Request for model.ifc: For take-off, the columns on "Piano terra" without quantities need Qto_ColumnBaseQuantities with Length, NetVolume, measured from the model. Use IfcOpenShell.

First a look at what the model holds.

```python
import ifcopenshell
import ifcopenshell.util.element
import ifcopenshell.util.unit

model = ifcopenshell.open("model.ifc")
print(model.schema)
for unit_type in ("LENGTHUNIT", "AREAUNIT", "VOLUMEUNIT"):
    print(unit_type, ifcopenshell.util.unit.calculate_unit_scale(model, unit_type))
storey = next(s for s in model.by_type("IfcBuildingStorey") if s.Name == "Piano terra")
columns = [e for e in ifcopenshell.util.element.get_decomposition(storey) if e.is_a("IfcColumn")]
for e in sorted(columns, key=lambda e: e.id()):
    print(e.id(), e.is_a(), e.Name, list(ifcopenshell.util.element.get_psets(e, qtos_only=True)), sep=" | ")
```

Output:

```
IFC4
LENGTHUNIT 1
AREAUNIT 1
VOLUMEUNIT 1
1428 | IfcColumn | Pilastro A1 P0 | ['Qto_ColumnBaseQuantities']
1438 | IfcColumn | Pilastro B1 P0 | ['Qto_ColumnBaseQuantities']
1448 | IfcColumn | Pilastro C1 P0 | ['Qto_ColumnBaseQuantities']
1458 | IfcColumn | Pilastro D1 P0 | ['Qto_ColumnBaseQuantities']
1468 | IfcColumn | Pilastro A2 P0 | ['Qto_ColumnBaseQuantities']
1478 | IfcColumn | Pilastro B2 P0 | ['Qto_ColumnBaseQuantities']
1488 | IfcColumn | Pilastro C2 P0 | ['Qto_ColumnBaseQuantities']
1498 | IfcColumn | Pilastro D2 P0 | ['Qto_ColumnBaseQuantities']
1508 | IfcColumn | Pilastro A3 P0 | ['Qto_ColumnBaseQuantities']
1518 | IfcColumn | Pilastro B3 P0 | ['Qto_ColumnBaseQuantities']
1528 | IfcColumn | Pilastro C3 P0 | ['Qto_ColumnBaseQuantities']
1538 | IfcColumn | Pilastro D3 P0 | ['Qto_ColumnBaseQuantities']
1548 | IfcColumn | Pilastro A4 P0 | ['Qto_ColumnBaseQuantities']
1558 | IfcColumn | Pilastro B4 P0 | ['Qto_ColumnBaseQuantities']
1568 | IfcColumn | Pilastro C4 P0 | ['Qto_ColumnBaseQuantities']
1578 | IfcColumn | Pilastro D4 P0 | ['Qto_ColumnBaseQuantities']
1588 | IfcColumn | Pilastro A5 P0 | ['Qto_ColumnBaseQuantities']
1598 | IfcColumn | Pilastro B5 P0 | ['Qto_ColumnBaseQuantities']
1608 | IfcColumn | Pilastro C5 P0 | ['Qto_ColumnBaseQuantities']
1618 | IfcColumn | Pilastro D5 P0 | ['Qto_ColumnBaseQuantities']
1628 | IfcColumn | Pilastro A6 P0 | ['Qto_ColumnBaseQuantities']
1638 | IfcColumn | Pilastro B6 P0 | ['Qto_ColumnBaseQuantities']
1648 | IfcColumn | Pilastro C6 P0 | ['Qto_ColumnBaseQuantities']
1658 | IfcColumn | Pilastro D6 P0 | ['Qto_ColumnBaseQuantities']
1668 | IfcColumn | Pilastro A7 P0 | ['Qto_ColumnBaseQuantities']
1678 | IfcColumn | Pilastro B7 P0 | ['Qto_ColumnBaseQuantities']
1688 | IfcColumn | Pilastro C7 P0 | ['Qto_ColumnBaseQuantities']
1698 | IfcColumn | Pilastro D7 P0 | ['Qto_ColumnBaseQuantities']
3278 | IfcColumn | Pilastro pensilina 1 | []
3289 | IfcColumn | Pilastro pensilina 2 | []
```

```python
import ifcopenshell
import ifcopenshell.api.pset
import ifcopenshell.geom
import ifcopenshell.util.element
import ifcopenshell.util.shape
import ifcopenshell.util.unit

model = ifcopenshell.open("model.ifc")
unit_scale = ifcopenshell.util.unit.calculate_unit_scale(model)
volume_scale = ifcopenshell.util.unit.calculate_unit_scale(model, "VOLUMEUNIT")
settings = ifcopenshell.geom.settings()

storey = next(s for s in model.by_type("IfcBuildingStorey") if s.Name == "Piano terra")
columns = [e for e in ifcopenshell.util.element.get_decomposition(storey) if e.is_a("IfcColumn")]

for e in sorted(columns, key=lambda e: e.id()):
    if ifcopenshell.util.element.get_psets(e, qtos_only=True, should_inherit=False):
        continue
    # Geometry comes back in metres, in the element's own axes.
    shape = ifcopenshell.geom.create_shape(settings, e)
    values = {
        "Length": ifcopenshell.util.shape.get_z(shape.geometry) / unit_scale,
        "NetVolume": ifcopenshell.util.shape.get_volume(shape.geometry) / volume_scale,
    }
    qto = ifcopenshell.api.pset.add_qto(model, product=e, name="Qto_ColumnBaseQuantities")
    ifcopenshell.api.pset.edit_qto(model, qto=qto, properties=values)
    print(e.id(), {k: round(v, 3) for k, v in values.items()})

model.write("model_v2.ifc")
```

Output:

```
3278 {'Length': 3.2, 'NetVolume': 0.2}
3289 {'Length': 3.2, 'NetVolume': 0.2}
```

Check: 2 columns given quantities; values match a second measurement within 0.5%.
